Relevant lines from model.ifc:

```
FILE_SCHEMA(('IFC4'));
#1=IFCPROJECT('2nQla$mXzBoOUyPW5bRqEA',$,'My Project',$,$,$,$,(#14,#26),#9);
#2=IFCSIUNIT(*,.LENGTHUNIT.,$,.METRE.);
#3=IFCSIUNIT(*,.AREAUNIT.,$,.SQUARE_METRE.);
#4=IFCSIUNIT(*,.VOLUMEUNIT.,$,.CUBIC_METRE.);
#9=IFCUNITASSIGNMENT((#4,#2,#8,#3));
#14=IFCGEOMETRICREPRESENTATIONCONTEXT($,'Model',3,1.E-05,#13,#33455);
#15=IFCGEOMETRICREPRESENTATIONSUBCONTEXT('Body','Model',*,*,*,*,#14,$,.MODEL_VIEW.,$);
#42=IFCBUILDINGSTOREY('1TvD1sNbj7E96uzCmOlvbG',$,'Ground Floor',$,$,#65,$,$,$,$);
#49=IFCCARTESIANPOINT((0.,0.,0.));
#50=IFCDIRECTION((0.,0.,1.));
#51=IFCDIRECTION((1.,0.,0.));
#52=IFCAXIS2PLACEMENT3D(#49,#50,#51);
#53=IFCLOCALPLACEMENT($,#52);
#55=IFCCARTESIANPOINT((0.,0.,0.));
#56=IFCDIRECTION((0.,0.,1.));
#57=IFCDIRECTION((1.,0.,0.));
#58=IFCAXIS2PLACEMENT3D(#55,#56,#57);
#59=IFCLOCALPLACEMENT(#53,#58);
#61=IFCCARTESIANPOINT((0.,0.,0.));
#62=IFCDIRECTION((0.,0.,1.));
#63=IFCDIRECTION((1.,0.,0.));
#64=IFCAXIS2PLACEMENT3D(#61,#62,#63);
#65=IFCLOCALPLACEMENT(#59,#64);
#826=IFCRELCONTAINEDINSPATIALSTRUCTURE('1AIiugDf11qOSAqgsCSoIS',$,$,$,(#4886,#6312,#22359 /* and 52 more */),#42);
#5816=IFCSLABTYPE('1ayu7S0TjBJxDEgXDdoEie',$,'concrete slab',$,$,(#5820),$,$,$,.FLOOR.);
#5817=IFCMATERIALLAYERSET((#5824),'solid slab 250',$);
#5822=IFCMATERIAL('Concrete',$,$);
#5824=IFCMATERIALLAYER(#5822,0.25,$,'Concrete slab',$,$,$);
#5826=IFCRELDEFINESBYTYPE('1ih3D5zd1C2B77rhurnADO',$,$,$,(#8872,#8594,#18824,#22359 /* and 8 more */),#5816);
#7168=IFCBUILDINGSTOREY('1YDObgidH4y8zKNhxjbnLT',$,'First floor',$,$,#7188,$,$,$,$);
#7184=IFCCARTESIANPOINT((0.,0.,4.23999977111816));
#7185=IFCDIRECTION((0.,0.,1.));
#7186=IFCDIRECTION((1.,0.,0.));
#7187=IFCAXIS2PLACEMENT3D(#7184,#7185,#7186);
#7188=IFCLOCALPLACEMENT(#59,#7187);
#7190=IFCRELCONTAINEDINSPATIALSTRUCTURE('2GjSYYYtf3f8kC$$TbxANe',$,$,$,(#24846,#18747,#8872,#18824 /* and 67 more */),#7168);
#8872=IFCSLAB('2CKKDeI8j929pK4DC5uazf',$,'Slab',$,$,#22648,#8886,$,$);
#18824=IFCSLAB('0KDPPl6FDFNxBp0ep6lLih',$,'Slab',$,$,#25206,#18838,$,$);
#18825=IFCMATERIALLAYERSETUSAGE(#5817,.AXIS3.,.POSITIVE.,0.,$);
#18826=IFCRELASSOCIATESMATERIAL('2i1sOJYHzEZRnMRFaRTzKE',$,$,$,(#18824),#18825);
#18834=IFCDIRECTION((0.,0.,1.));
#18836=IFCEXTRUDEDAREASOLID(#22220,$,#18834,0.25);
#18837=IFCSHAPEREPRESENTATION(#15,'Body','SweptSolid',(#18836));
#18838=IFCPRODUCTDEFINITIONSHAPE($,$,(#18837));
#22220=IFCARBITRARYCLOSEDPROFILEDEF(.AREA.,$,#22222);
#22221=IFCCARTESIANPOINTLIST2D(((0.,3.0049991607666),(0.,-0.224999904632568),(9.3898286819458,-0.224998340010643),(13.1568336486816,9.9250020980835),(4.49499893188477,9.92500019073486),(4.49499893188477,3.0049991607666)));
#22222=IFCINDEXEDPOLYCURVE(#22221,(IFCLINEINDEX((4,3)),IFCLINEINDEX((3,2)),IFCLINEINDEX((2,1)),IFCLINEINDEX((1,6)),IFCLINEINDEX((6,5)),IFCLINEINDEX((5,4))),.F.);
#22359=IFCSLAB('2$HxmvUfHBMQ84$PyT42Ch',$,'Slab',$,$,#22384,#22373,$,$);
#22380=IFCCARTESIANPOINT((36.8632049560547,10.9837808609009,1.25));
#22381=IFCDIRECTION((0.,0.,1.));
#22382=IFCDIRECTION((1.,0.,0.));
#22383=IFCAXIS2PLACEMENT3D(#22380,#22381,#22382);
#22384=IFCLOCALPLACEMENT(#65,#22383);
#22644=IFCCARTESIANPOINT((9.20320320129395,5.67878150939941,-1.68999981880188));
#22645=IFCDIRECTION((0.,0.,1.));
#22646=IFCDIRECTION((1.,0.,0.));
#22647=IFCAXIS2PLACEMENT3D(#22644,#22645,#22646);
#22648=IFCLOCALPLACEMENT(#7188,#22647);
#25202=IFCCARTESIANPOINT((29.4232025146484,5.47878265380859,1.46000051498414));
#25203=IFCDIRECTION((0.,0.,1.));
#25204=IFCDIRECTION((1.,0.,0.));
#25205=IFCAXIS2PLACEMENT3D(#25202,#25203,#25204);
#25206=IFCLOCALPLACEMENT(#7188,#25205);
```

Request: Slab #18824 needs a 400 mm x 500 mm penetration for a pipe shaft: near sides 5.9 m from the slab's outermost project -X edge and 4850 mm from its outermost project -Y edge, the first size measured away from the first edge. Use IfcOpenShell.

```python
import numpy as np
import ifcopenshell
import ifcopenshell.api.feature
import ifcopenshell.api.geometry
import ifcopenshell.api.root
import ifcopenshell.geom
import ifcopenshell.util.placement
import ifcopenshell.util.representation
import ifcopenshell.util.shape
import ifcopenshell.util.unit

model = ifcopenshell.open("model.ifc")
unit_scale = ifcopenshell.util.unit.calculate_unit_scale(model)
settings = ifcopenshell.geom.settings()


def volume(element):
    """Net volume in cubic metres, openings subtracted."""
    shape = ifcopenshell.geom.create_shape(settings, element)
    return ifcopenshell.util.shape.get_volume(shape.geometry)


slab = model.by_id(18824)
before = volume(slab)

# Extent in the slab's own axes, in metres. The edges named are its -X and -Y sides.
slab_shape = ifcopenshell.geom.create_shape(settings, slab)
vertices = ifcopenshell.util.shape.get_vertices(slab_shape.geometry)
x_min, y_min, bottom = vertices.min(axis=0)
top = vertices[:, 2].max()

opening = ifcopenshell.api.root.create_entity(model, ifc_class="IfcOpeningElement", name="Pipe shaft opening", predefined_type="OPENING")
context = ifcopenshell.util.representation.get_context(model, "Model", "Body", "MODEL_VIEW")
width, depth = 0.4, 0.5
outline = [(0.0, 0.0), (width, 0.0), (width, depth), (0.0, depth), (0.0, 0.0)]
# Overshoot both faces by 50 mm so the cut is clean.
shape = ifcopenshell.api.geometry.add_slab_representation(
    model, context=context, depth=top - bottom + 0.1, polyline=outline
)
ifcopenshell.api.geometry.assign_representation(model, product=opening, representation=shape)

matrix = ifcopenshell.util.placement.get_local_placement(slab.ObjectPlacement)
matrix[:, 3] = matrix @ np.append(np.array([x_min + 5.9, y_min + 4.85, bottom - 0.05]) / unit_scale, 1.0)
ifcopenshell.api.geometry.edit_object_placement(model, product=opening, matrix=matrix, is_si=False)
ifcopenshell.api.feature.add_feature(model, feature=opening, element=slab)

after = volume(slab)

print(f"slab volume {before:.3f} -> {after:.3f} m3")

model.write("model_edited.ifc")
```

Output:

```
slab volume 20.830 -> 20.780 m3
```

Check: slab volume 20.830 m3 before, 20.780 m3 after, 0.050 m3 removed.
